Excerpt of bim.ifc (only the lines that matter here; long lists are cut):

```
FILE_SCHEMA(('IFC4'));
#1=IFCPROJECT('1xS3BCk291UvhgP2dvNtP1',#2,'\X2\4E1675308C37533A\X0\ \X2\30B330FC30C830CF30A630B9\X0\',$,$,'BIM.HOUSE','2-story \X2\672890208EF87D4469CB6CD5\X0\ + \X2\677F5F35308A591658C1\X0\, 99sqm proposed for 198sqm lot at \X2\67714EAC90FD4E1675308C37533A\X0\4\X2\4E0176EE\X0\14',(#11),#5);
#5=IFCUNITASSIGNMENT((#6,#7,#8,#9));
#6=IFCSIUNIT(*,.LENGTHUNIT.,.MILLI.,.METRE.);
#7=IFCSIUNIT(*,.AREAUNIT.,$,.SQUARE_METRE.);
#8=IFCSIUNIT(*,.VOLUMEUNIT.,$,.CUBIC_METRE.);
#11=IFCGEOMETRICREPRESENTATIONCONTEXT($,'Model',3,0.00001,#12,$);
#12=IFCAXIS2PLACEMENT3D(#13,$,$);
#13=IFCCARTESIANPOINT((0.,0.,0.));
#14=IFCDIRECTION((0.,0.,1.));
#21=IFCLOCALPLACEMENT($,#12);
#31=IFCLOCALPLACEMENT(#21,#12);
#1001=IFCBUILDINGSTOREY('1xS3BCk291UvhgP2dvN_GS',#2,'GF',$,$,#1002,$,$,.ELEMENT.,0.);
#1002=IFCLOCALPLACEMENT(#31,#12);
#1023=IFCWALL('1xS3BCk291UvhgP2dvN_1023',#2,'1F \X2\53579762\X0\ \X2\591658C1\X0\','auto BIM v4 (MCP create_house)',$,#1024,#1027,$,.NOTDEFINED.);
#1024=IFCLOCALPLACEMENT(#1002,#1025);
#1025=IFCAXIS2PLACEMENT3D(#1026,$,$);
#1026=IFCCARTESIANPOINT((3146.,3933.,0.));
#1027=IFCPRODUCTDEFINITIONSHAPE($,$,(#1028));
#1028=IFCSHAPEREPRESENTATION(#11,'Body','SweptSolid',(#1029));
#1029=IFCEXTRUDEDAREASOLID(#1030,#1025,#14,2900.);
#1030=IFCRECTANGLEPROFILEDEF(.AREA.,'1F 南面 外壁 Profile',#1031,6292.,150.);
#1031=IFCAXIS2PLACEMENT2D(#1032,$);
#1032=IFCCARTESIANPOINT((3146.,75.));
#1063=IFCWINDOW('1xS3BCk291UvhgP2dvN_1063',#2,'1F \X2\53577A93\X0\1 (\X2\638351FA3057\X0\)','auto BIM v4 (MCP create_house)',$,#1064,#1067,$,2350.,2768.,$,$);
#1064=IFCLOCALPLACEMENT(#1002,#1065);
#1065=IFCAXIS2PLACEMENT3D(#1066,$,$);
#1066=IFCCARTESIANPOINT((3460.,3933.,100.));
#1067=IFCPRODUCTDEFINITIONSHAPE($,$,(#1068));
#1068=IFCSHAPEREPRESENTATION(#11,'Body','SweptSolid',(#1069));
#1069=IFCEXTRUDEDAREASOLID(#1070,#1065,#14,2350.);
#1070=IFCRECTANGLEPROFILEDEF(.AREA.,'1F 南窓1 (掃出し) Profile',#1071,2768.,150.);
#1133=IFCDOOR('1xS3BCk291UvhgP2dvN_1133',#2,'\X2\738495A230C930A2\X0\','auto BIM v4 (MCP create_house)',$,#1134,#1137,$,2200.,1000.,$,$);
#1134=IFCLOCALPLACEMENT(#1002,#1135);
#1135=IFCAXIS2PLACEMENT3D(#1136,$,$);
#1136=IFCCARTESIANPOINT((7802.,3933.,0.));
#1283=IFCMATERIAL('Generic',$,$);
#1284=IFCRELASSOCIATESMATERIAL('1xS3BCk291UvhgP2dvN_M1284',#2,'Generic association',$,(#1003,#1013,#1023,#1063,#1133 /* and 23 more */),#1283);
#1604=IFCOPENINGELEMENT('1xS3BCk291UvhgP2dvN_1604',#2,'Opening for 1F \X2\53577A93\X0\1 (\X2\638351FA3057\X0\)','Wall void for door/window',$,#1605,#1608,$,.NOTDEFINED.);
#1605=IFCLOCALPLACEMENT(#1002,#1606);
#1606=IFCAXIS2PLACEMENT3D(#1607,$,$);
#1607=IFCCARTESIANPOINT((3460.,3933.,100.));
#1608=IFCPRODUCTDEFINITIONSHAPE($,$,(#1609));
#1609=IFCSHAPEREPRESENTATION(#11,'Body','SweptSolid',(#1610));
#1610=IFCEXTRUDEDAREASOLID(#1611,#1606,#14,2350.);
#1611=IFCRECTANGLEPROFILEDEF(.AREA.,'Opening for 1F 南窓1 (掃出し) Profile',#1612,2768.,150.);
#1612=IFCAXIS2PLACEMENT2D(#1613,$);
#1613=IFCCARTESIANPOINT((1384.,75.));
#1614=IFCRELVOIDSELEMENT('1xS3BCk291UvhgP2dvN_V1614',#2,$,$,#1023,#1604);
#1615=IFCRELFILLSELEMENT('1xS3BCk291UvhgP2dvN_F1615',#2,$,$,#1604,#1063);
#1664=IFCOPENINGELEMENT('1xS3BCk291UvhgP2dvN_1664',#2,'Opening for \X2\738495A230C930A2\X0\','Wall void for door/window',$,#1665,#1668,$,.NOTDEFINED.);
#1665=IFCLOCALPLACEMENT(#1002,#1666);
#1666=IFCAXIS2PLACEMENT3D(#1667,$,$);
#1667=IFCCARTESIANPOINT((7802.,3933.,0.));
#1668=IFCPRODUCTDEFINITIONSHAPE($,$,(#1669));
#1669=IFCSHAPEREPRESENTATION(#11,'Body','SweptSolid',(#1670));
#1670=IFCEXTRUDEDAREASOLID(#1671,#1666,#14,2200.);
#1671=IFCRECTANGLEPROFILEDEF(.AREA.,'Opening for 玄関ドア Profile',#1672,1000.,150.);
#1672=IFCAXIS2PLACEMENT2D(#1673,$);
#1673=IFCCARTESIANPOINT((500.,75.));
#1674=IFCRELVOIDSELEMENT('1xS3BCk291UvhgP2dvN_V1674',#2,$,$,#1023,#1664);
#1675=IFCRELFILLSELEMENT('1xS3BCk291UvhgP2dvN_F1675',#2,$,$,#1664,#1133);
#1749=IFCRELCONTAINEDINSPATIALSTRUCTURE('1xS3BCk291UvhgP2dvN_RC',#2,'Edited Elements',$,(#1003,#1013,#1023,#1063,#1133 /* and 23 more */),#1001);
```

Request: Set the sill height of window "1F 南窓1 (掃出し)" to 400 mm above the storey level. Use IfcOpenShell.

```python
import numpy as np
import ifcopenshell
import ifcopenshell.api.geometry
import ifcopenshell.geom
import ifcopenshell.util.element
import ifcopenshell.util.placement
import ifcopenshell.util.shape
import ifcopenshell.util.unit

model = ifcopenshell.open("bim.ifc")
unit_scale = ifcopenshell.util.unit.calculate_unit_scale(model)

window = model.by_id(1063)
opening = window.FillsVoids[0].RelatingOpeningElement
storey = ifcopenshell.util.element.get_container(window, ifc_class="IfcBuildingStorey")
level = ifcopenshell.util.placement.get_local_placement(storey.ObjectPlacement)[2, 3]

# The opening's origin need not be at the sill, so measure its lowest point.
shape = ifcopenshell.geom.create_shape(ifcopenshell.geom.settings(), opening)
bottom = ifcopenshell.util.shape.get_shape_bottom_elevation(shape, shape.geometry) / unit_scale
dz = level + 0.4 / unit_scale - bottom

shift = np.array([0.0, 0.0, dz])
# The window is not placed relative to its opening, so move both.
for product in (opening, window):
    matrix = ifcopenshell.util.placement.get_local_placement(product.ObjectPlacement)
    matrix[:3, 3] += shift
    ifcopenshell.api.geometry.edit_object_placement(model, product=product, matrix=matrix, is_si=False)

print(f"moved by {dz * unit_scale:+.3f} m")

model.write("bim_v2.ifc")
```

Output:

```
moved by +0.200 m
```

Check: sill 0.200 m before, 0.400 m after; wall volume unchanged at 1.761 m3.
